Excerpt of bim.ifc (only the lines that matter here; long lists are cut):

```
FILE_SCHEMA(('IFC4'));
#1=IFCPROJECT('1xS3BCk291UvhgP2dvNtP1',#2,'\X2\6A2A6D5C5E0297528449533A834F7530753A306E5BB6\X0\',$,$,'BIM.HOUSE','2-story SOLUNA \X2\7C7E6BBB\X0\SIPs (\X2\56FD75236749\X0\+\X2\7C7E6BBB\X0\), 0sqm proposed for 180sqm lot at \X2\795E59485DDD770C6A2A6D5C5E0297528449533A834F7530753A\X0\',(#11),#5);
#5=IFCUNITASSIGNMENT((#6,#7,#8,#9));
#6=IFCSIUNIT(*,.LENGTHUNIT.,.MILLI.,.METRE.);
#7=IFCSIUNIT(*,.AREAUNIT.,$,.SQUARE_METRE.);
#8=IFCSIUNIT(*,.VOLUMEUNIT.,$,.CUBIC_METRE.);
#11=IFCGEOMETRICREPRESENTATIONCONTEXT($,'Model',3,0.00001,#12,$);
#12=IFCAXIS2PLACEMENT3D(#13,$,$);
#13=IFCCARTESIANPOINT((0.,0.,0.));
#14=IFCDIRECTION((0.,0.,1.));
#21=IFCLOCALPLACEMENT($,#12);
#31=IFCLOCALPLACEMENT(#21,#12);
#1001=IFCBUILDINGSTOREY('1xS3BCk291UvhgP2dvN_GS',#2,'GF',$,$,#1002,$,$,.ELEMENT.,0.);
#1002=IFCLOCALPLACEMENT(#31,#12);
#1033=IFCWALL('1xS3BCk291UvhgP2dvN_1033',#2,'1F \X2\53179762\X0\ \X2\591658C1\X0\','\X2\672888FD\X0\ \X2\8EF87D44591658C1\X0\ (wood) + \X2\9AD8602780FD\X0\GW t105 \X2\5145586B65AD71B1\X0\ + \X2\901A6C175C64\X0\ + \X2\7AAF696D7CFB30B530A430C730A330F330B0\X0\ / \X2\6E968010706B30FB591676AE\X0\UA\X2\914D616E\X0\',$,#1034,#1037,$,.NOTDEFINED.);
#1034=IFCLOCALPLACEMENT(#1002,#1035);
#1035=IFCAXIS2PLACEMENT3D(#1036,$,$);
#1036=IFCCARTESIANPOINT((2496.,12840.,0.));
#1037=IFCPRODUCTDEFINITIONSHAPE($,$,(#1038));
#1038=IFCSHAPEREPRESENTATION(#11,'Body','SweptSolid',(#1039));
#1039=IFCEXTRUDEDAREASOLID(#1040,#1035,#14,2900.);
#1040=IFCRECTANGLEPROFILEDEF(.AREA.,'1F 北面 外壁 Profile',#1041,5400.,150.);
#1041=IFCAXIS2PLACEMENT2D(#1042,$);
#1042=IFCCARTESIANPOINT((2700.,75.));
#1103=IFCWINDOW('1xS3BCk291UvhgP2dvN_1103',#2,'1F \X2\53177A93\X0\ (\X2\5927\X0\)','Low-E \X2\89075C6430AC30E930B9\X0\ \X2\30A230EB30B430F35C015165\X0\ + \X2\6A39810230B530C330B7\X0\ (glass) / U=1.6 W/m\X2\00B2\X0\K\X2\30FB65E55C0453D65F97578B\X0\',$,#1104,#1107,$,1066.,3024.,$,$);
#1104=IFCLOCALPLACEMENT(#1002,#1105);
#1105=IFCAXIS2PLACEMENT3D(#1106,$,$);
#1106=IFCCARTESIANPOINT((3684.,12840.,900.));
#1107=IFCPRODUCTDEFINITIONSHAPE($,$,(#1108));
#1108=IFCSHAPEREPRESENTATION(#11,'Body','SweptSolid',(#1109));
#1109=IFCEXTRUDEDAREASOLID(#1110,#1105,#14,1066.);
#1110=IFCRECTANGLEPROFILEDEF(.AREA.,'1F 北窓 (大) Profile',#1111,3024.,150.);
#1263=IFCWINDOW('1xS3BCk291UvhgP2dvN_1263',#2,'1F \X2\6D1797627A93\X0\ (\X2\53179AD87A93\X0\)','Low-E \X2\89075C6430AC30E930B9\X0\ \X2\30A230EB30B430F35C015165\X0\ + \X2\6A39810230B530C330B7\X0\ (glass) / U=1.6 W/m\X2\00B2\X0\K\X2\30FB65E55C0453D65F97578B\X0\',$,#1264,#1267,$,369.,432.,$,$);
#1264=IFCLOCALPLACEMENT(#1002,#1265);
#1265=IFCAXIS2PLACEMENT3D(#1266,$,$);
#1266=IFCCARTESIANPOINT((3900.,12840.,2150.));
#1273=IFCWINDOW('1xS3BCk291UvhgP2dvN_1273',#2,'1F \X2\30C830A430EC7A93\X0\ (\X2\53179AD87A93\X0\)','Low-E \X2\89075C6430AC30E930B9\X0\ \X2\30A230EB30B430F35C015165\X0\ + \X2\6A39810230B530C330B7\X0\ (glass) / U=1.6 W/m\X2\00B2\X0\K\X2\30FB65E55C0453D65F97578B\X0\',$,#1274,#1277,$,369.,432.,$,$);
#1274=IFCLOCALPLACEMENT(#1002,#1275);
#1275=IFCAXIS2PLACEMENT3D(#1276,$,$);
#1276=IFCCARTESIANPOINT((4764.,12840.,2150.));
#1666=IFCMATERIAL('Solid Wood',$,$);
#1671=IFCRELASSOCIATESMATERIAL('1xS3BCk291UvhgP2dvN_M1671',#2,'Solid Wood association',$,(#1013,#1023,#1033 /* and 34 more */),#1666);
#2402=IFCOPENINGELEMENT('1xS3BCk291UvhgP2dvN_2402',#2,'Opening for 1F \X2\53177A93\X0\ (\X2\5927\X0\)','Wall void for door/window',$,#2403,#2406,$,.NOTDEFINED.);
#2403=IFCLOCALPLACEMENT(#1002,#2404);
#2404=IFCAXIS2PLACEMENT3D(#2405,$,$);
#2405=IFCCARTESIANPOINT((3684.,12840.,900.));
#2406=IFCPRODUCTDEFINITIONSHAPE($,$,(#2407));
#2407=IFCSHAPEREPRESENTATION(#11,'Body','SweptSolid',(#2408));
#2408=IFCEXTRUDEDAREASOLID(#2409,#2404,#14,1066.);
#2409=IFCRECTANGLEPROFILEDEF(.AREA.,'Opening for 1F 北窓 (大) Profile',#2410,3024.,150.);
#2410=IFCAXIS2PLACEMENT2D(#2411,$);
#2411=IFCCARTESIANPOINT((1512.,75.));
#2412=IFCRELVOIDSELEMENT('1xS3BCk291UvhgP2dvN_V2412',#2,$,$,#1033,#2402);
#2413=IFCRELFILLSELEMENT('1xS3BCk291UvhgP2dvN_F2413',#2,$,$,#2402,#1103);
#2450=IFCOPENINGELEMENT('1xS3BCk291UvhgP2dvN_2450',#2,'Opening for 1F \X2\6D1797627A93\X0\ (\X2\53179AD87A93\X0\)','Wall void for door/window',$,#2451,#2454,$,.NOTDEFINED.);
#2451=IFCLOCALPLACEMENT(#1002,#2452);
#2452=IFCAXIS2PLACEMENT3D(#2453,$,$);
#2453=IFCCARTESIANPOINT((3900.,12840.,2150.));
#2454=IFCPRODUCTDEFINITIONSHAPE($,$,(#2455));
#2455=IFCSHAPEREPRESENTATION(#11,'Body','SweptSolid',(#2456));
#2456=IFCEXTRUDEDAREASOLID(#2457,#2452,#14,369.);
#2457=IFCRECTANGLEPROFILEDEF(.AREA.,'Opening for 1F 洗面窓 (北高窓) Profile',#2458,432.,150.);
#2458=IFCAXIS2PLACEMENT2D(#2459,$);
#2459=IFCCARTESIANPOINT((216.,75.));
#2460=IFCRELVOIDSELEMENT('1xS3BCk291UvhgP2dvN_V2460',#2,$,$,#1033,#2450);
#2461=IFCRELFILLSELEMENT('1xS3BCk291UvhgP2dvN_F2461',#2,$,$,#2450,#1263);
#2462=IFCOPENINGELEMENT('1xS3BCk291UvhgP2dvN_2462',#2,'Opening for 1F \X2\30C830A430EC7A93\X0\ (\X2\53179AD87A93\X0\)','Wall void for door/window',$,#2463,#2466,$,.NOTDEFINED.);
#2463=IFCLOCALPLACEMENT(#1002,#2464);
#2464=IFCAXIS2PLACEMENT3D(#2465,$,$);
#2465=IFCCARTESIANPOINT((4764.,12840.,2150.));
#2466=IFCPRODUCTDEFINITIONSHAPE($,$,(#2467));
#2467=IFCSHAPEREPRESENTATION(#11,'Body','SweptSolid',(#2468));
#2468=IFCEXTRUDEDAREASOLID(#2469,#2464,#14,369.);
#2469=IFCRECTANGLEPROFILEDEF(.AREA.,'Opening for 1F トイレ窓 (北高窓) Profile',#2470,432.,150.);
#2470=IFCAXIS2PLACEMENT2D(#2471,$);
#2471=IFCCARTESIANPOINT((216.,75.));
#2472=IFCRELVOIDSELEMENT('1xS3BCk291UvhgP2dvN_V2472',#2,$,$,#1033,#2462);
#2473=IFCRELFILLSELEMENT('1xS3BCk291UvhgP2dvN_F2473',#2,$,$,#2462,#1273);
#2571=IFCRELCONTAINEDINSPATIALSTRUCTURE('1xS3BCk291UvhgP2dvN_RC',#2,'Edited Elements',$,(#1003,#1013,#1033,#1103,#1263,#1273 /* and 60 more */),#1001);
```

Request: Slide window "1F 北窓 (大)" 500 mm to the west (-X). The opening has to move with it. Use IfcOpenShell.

```python
import ifcopenshell
import ifcopenshell.api.geometry
import ifcopenshell.util.placement

model = ifcopenshell.open("bim.ifc")

window = model.by_guid("1xS3BCk291UvhgP2dvN_1103")
opening = window.FillsVoids[0].RelatingOpeningElement
wall = opening.VoidsElements[0].RelatingBuildingElement

wall_matrix = ifcopenshell.util.placement.get_local_placement(wall.ObjectPlacement)
shift = wall_matrix[:3, 0] * -500.0
before = ifcopenshell.util.placement.get_local_placement(window.ObjectPlacement)[:3, 3].copy()

# The window is not placed relative to its opening, so move both.
for product in (opening, window):
    matrix = ifcopenshell.util.placement.get_local_placement(product.ObjectPlacement)
    matrix[:3, 3] += shift
    ifcopenshell.api.geometry.edit_object_placement(model, product=product, matrix=matrix, is_si=False)

after = ifcopenshell.util.placement.get_local_placement(window.ObjectPlacement)[:3, 3]
print("window moved by", (after - before).round(3) + 0.0)

model.write("bim_edited.ifc")
```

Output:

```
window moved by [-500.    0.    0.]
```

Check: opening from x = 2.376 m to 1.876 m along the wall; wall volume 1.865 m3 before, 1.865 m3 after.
